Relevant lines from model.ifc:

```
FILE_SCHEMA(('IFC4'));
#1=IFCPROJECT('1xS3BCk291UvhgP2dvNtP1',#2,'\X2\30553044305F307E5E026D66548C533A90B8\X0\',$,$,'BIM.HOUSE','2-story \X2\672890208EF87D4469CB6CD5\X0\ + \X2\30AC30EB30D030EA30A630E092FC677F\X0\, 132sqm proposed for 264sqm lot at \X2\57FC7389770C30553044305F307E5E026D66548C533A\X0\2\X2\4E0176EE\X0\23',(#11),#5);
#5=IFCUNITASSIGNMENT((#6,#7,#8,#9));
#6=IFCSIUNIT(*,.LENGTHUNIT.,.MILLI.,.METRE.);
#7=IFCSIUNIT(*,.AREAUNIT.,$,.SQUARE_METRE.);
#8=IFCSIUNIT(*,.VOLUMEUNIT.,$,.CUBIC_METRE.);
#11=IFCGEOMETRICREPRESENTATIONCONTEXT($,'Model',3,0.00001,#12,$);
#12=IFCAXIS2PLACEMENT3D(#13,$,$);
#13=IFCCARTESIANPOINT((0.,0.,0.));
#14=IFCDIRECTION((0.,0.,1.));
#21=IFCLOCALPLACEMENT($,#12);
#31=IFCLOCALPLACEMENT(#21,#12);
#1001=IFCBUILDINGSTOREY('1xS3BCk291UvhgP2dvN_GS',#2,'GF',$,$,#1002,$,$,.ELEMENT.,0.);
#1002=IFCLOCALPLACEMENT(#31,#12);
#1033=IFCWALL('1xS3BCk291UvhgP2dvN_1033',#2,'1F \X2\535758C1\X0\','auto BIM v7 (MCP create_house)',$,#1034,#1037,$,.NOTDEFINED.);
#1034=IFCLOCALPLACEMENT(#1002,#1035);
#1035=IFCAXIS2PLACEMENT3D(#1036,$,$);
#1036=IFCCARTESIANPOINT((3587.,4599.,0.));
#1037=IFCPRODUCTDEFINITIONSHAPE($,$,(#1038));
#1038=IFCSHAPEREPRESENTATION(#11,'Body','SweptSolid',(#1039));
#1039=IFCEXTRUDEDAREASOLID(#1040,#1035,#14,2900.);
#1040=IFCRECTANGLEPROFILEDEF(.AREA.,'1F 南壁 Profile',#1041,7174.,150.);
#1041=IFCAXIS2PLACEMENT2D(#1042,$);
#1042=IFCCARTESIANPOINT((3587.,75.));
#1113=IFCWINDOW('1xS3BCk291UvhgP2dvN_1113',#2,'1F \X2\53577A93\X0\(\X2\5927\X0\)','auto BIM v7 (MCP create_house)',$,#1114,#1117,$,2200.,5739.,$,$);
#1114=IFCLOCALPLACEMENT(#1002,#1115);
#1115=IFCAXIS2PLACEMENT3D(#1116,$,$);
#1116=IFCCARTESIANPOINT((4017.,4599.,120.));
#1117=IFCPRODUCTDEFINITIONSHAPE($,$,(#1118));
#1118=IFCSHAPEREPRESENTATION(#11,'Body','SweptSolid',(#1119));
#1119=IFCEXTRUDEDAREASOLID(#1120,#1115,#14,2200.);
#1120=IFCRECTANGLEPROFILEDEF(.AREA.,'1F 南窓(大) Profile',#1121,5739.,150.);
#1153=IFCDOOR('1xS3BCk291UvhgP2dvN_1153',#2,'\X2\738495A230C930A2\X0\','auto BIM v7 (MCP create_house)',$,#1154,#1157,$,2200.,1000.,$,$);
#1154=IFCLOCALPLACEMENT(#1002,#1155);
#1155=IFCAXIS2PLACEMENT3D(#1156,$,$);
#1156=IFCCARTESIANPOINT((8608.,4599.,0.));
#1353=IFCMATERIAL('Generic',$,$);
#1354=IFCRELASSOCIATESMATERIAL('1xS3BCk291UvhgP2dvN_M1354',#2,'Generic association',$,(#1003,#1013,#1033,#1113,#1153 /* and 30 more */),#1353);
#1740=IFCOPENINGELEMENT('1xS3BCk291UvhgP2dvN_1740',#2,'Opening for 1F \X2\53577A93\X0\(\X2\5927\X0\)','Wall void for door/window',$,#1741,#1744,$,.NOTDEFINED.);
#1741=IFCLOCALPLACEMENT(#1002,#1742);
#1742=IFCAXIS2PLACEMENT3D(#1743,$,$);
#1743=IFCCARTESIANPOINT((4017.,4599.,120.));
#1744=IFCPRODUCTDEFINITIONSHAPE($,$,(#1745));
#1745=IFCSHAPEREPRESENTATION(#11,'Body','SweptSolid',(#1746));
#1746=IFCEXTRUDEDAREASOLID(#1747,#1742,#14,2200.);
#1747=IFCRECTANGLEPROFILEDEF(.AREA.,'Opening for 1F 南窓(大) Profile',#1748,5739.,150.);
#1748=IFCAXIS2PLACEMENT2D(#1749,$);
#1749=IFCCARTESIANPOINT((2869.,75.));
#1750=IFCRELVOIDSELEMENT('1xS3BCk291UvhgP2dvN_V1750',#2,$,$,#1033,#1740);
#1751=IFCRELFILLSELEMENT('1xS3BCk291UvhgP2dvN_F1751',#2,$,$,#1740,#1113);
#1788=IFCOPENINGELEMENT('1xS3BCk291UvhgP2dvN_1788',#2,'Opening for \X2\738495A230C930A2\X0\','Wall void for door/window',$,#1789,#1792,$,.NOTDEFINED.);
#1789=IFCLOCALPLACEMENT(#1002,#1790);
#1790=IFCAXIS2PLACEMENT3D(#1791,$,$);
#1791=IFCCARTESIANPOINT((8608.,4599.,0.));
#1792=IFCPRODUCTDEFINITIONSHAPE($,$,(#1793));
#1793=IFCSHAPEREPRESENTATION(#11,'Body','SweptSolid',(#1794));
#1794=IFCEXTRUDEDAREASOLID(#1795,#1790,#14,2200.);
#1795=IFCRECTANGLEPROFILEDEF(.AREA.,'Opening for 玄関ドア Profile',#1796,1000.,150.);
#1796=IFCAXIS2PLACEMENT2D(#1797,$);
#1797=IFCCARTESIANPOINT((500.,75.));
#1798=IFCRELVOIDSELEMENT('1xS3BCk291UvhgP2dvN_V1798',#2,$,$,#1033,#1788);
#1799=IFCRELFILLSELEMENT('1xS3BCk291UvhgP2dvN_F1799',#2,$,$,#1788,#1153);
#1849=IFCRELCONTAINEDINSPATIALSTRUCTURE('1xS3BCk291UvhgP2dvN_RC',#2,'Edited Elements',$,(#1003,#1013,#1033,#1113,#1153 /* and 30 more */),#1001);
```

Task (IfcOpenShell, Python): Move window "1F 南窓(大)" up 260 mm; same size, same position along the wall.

```python
import numpy as np
import ifcopenshell
import ifcopenshell.api.geometry
import ifcopenshell.util.placement
import ifcopenshell.util.unit

model = ifcopenshell.open("model.ifc")
unit_scale = ifcopenshell.util.unit.calculate_unit_scale(model)

window = model.by_id(1113)
opening = window.FillsVoids[0].RelatingOpeningElement
dz = 0.26 / unit_scale

shift = np.array([0.0, 0.0, dz])
# The window is not placed relative to its opening, so move both.
for product in (opening, window):
    matrix = ifcopenshell.util.placement.get_local_placement(product.ObjectPlacement)
    matrix[:3, 3] += shift
    ifcopenshell.api.geometry.edit_object_placement(model, product=product, matrix=matrix, is_si=False)

print(f"moved by {dz * unit_scale:+.3f} m")

model.write("model_updated.ifc")
```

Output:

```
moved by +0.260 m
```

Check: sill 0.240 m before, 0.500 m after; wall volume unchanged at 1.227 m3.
